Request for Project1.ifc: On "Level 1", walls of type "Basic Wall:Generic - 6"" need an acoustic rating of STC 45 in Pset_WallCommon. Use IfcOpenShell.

First a look at what the model holds.

```python
import ifcopenshell
import ifcopenshell.util.element

model = ifcopenshell.open("Project1.ifc")
print(model.schema)
storey = next(s for s in model.by_type("IfcBuildingStorey") if s.Name == "Level 1")
walls = [e for e in ifcopenshell.util.element.get_decomposition(storey) if e.is_a("IfcWall")]
seen = {}
for e in walls:
    element_type = ifcopenshell.util.element.get_type(e)
    key = (element_type.Name if element_type != e and element_type else None, ifcopenshell.util.element.get_pset(e, "Pset_WallCommon", "AcousticRating"))
    seen[key] = seen.get(key, 0) + 1
for (name, value), count in sorted(seen.items(), key=str):
    print(count, "x", name, "|", value)
```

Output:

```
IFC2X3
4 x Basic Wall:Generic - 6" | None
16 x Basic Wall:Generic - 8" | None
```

```python
import ifcopenshell
import ifcopenshell.api.pset
import ifcopenshell.util.element

model = ifcopenshell.open("Project1.ifc")

storey = next(s for s in model.by_type("IfcBuildingStorey") if s.Name == "Level 1")
walls = [e for e in ifcopenshell.util.element.get_decomposition(storey) if e.is_a("IfcWall")]

count = 0
for e in walls:
    element_type = ifcopenshell.util.element.get_type(e)
    if element_type in (None, e) or element_type.Name != 'Basic Wall:Generic - 6"':
        continue
    # add_pset returns the element's existing set when there is one.
    pset = ifcopenshell.api.pset.add_pset(model, product=e, name="Pset_WallCommon")
    ifcopenshell.api.pset.edit_pset(model, pset=pset, properties={"AcousticRating": "STC 45"})
    count += 1

print(count, "walls updated")

model.write("Project1_rev.ifc")
```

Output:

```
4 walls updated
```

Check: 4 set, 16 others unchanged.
